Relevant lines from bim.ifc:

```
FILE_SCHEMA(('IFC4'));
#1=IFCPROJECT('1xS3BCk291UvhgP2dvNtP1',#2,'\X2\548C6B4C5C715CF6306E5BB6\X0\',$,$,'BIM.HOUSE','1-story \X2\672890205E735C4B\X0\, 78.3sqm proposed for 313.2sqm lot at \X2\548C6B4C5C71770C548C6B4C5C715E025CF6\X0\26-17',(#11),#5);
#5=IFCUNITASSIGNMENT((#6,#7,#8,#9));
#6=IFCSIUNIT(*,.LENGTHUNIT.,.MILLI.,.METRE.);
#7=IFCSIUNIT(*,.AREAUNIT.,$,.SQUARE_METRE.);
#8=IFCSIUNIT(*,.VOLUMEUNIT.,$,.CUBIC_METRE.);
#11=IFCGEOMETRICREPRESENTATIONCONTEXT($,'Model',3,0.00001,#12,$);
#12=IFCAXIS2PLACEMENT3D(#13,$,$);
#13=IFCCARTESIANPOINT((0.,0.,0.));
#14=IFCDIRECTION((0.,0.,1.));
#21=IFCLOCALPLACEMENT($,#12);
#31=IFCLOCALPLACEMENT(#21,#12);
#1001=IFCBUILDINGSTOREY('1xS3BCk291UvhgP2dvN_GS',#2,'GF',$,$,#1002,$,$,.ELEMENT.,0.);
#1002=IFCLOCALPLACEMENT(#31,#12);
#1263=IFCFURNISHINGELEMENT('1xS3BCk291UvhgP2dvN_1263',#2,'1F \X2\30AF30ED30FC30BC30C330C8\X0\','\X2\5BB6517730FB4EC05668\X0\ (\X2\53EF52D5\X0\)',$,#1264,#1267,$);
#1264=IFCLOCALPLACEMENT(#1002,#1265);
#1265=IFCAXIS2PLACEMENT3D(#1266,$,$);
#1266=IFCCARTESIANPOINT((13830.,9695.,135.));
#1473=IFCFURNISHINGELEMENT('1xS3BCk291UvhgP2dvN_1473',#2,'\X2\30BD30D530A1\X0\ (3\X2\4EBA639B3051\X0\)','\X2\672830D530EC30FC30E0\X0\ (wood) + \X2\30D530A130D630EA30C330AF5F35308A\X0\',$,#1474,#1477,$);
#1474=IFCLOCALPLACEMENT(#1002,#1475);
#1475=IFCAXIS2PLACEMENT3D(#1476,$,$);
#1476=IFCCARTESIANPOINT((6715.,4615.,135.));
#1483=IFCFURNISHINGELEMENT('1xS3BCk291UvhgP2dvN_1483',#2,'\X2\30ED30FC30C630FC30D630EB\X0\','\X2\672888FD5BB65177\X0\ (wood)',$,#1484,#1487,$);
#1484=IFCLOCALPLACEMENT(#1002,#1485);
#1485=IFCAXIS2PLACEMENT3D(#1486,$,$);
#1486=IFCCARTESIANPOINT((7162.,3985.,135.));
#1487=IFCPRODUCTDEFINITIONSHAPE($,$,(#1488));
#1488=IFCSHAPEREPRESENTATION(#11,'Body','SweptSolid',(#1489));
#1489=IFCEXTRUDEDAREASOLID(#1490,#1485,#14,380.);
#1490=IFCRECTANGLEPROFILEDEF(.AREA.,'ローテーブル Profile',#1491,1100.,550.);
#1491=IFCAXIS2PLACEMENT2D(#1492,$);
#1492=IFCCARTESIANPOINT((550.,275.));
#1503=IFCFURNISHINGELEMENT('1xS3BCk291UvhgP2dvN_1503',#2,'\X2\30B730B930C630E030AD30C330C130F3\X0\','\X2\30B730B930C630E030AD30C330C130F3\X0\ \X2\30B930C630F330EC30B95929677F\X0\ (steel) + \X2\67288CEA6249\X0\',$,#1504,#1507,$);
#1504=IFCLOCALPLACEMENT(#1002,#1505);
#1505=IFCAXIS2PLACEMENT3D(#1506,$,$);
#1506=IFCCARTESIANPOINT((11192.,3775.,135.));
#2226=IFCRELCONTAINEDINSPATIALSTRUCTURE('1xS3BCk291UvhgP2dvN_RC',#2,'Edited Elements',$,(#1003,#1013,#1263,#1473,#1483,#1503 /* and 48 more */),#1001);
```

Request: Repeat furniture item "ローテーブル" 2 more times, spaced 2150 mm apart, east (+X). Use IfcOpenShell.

```python
import numpy as np
import ifcopenshell
import ifcopenshell.api.geometry
import ifcopenshell.api.root
import ifcopenshell.util.element
import ifcopenshell.util.placement

model = ifcopenshell.open("bim.ifc")


def reuse_history(source, copy):
    """copy_class also copies each property set's owner history, people and application; keep the originals."""
    for rel in copy.IsDefinedBy:
        if rel.is_a("IfcRelDefinesByProperties") and (history := rel.RelatingPropertyDefinition.OwnerHistory):
            rel.RelatingPropertyDefinition.OwnerHistory = source.OwnerHistory
            ifcopenshell.util.element.remove_deep2(model, history)


source = model.by_guid("1xS3BCk291UvhgP2dvN_1483")
base = ifcopenshell.util.placement.get_local_placement(source.ObjectPlacement)
step = np.array([1.0, 0.0, 0.0]) * 2150.0

for i in range(1, 3):
    copy = ifcopenshell.api.root.copy_class(model, product=source)
    copy.Representation = ifcopenshell.util.element.copy_deep(
        model, source.Representation, exclude=["IfcGeometricRepresentationContext", "IfcRepresentationMap"]
    )
    reuse_history(source, copy)
    matrix = base.copy()
    matrix[:3, 3] += i * step
    print("added at", matrix[:3, 3].round(3) + 0.0)
    ifcopenshell.api.geometry.edit_object_placement(model, product=copy, matrix=matrix, is_si=False)

model.write("bim_rev.ifc")
```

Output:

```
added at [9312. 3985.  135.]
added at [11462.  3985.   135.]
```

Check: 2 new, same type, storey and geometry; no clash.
